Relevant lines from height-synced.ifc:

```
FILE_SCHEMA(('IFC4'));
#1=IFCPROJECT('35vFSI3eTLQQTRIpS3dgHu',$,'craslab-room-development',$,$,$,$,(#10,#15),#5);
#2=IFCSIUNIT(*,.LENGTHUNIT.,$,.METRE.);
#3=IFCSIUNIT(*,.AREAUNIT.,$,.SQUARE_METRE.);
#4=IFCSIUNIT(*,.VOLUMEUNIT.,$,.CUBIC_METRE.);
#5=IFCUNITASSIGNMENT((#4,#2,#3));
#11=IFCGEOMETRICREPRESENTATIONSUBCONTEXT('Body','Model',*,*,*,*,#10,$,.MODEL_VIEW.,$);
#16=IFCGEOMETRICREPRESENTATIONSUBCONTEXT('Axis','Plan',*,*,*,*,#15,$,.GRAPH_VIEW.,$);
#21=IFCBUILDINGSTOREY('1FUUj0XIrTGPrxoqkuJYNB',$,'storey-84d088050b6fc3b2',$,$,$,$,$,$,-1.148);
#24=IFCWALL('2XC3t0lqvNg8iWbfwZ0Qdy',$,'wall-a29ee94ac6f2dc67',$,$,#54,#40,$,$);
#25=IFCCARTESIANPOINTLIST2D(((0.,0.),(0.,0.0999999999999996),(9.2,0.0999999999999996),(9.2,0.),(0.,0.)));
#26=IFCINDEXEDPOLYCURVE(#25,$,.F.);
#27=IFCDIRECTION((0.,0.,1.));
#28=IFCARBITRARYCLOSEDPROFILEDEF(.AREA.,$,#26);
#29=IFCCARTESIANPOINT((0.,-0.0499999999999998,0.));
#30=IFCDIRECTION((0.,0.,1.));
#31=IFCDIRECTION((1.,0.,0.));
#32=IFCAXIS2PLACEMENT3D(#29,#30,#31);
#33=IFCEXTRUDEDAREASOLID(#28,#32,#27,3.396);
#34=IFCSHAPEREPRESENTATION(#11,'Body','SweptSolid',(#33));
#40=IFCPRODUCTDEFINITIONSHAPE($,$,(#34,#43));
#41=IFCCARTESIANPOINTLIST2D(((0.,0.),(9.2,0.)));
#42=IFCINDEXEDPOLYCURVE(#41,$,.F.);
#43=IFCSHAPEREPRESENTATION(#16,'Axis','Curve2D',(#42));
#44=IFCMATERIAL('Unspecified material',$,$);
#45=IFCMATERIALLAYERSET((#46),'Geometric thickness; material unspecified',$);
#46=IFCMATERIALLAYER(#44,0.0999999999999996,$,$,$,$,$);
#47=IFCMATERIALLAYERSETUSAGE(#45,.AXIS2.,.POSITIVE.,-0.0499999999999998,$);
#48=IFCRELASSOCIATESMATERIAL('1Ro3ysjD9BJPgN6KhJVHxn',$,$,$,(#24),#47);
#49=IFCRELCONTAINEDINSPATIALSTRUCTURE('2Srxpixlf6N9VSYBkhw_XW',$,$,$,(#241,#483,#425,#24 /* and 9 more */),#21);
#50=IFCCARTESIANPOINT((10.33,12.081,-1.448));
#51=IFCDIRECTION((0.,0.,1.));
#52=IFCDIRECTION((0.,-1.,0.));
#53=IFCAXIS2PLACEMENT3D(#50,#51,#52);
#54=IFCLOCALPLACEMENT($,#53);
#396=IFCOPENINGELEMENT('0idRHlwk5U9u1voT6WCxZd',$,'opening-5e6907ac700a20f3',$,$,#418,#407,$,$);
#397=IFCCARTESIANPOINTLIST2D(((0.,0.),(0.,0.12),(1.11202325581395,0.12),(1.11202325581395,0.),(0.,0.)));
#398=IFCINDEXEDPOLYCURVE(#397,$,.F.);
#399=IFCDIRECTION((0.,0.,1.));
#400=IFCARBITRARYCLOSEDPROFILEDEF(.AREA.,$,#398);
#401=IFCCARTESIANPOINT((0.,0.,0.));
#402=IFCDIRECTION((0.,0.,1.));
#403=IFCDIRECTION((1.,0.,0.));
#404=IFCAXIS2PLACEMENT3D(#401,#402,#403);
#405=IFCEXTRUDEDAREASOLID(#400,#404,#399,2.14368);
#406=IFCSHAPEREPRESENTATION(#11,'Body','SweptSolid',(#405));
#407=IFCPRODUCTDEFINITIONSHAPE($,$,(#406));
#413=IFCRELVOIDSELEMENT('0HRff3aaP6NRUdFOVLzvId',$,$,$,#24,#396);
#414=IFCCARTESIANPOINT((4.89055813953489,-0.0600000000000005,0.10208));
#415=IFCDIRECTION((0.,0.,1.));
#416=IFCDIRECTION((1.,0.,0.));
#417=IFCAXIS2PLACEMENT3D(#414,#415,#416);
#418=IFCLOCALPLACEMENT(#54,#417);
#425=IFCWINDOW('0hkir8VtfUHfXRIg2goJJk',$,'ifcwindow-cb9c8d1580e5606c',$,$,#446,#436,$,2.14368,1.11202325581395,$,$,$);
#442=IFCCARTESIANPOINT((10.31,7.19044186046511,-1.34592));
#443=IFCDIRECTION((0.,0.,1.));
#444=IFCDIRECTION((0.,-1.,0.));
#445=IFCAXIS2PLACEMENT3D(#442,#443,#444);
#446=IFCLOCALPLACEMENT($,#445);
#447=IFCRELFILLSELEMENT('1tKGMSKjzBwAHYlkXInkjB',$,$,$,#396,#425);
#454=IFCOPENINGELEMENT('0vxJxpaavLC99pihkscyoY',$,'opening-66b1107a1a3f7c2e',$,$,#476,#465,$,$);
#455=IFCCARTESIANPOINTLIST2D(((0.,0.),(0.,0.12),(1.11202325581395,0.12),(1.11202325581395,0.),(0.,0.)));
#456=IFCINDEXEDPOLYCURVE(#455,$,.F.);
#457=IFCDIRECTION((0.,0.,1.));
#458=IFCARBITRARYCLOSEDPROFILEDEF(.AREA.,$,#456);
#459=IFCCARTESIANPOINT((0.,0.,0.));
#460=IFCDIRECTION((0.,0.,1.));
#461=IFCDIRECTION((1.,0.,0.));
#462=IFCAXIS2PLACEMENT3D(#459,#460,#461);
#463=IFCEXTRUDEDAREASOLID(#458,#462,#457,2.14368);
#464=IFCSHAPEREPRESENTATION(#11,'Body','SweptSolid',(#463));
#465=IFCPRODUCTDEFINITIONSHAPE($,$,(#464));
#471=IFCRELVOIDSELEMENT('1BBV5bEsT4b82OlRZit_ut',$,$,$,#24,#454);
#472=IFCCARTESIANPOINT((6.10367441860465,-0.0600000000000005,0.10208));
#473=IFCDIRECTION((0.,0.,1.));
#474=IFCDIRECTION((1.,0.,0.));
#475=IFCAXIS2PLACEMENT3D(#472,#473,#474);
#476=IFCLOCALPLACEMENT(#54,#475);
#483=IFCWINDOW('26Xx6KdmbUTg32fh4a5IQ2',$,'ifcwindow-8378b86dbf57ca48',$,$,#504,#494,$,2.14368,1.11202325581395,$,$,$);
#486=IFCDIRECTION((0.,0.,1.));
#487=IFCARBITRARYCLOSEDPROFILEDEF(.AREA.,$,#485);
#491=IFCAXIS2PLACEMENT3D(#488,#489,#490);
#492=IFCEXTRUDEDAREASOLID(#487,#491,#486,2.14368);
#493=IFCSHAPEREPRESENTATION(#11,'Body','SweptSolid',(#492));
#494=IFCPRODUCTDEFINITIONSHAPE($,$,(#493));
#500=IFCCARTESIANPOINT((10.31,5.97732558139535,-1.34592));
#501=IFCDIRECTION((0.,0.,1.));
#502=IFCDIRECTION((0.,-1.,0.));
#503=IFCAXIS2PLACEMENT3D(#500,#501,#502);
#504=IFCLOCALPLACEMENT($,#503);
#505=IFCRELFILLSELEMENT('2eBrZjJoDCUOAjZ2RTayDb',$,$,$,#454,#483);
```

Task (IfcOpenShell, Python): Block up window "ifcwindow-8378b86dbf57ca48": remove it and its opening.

```python
import ifcopenshell
import ifcopenshell.api.feature
import ifcopenshell.api.root
import ifcopenshell.geom
import ifcopenshell.util.shape

model = ifcopenshell.open("height-synced.ifc")
settings = ifcopenshell.geom.settings()


def volume(element):
    """Net volume in cubic metres, openings subtracted."""
    shape = ifcopenshell.geom.create_shape(settings, element)
    return ifcopenshell.util.shape.get_volume(shape.geometry)


window = model.by_guid("26Xx6KdmbUTg32fh4a5IQ2")
opening = window.FillsVoids[0].RelatingOpeningElement
wall = opening.VoidsElements[0].RelatingBuildingElement
before = volume(wall)

ifcopenshell.api.root.remove_product(model, product=window)
ifcopenshell.api.feature.remove_feature(model, feature=opening)

after = volume(wall)

print(f"wall volume {before:.3f} -> {after:.3f} m3")

model.write("height-synced_edited.ifc")
```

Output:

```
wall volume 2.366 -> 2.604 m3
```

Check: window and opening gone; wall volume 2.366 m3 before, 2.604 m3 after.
